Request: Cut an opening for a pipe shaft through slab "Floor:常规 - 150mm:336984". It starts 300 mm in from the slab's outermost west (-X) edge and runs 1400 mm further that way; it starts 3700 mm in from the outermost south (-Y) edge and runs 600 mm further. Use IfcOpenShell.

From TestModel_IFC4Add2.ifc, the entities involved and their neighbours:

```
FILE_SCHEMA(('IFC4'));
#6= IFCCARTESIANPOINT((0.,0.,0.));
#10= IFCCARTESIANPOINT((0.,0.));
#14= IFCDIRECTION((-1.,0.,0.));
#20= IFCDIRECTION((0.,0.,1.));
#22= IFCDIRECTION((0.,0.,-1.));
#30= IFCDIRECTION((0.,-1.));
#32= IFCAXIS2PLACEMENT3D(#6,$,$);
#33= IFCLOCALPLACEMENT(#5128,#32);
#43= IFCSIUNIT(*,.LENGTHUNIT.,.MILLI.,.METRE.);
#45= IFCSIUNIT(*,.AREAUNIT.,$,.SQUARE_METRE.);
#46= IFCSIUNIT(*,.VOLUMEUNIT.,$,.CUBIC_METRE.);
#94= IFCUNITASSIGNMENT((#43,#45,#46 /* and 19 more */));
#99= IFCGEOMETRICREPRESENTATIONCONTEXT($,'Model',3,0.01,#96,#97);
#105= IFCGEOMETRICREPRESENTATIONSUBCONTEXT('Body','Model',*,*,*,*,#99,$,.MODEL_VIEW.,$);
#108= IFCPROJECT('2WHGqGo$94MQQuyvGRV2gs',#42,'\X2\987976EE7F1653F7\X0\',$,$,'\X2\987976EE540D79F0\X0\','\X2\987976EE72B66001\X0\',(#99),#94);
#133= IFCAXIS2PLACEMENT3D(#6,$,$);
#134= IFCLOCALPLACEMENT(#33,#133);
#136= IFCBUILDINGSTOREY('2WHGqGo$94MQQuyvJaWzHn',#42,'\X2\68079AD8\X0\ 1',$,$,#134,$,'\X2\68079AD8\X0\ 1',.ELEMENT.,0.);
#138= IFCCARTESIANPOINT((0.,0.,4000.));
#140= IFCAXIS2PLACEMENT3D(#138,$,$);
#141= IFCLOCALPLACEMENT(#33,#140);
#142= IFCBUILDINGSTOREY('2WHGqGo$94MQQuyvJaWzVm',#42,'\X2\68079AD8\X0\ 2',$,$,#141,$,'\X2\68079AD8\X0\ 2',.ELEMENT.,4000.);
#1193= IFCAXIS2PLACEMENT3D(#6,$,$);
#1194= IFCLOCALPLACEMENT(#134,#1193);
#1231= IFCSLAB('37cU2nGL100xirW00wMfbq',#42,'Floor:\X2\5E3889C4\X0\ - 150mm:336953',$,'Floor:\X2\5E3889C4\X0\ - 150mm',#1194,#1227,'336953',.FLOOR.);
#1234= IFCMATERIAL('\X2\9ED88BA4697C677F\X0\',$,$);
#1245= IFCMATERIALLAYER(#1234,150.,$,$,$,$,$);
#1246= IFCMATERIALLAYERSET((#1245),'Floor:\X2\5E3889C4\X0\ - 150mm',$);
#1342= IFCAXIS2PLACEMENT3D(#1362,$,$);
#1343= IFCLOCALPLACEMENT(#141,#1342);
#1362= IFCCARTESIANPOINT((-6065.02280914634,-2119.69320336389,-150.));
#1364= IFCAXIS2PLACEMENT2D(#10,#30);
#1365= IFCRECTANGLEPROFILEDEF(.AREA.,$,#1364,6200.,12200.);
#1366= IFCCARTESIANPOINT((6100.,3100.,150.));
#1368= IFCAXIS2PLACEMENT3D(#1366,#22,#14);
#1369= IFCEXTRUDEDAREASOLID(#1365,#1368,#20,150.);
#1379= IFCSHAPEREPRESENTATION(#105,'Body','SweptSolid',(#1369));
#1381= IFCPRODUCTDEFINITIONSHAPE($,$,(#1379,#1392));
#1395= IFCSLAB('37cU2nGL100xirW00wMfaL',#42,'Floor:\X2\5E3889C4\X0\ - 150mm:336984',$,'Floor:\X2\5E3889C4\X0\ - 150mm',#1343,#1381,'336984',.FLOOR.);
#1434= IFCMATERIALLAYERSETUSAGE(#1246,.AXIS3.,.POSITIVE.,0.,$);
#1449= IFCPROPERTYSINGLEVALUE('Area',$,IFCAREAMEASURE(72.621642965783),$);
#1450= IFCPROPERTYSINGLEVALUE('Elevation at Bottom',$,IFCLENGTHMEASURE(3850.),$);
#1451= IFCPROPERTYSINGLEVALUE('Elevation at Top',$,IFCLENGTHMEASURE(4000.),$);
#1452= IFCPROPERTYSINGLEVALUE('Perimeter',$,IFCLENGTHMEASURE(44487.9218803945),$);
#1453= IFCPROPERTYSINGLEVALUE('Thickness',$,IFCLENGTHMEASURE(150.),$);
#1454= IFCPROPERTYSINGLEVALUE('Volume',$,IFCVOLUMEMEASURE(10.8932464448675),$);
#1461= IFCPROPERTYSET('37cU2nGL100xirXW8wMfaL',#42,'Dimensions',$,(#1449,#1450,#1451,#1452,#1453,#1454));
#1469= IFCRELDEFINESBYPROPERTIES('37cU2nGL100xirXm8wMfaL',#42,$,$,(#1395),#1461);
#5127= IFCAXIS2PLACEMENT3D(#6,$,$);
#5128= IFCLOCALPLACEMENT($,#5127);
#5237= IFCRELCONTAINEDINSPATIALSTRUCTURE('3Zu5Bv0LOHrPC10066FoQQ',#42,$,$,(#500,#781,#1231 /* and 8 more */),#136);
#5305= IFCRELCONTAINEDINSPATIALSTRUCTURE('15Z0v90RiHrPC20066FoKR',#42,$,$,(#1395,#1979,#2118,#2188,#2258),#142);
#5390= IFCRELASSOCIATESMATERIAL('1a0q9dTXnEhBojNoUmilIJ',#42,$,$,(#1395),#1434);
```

```python
import numpy as np
import ifcopenshell
import ifcopenshell.api.feature
import ifcopenshell.api.geometry
import ifcopenshell.api.pset
import ifcopenshell.api.root
import ifcopenshell.geom
import ifcopenshell.util.element
import ifcopenshell.util.placement
import ifcopenshell.util.representation
import ifcopenshell.util.shape
import ifcopenshell.util.unit

model = ifcopenshell.open("TestModel_IFC4Add2.ifc")
unit_scale = ifcopenshell.util.unit.calculate_unit_scale(model)
area_scale = ifcopenshell.util.unit.calculate_unit_scale(model, "AREAUNIT")
volume_scale = ifcopenshell.util.unit.calculate_unit_scale(model, "VOLUMEUNIT")
settings = ifcopenshell.geom.settings()


def volume(element):
    """Net volume in cubic metres, openings subtracted."""
    shape = ifcopenshell.geom.create_shape(settings, element)
    return ifcopenshell.util.shape.get_volume(shape.geometry)


slab = model.by_guid("37cU2nGL100xirW00wMfaL")
before = volume(slab)

# Extent in the slab's own axes, in metres. The edges named are its -X and -Y sides.
slab_shape = ifcopenshell.geom.create_shape(settings, slab)
vertices = ifcopenshell.util.shape.get_vertices(slab_shape.geometry)
x_min, y_min, bottom = vertices.min(axis=0)
top = vertices[:, 2].max()

opening = ifcopenshell.api.root.create_entity(model, ifc_class="IfcOpeningElement", name="Pipe shaft opening", predefined_type="OPENING")
context = ifcopenshell.util.representation.get_context(model, "Model", "Body", "MODEL_VIEW")
width, depth = 1.4, 0.6
outline = [(0.0, 0.0), (width, 0.0), (width, depth), (0.0, depth), (0.0, 0.0)]
# Overshoot both faces by 50 mm so the cut is clean.
shape = ifcopenshell.api.geometry.add_slab_representation(
    model, context=context, depth=top - bottom + 0.1, polyline=outline
)
ifcopenshell.api.geometry.assign_representation(model, product=opening, representation=shape)

matrix = ifcopenshell.util.placement.get_local_placement(slab.ObjectPlacement)
matrix[:, 3] = matrix @ np.append(np.array([x_min + 0.3, y_min + 3.7, bottom - 0.05]) / unit_scale, 1.0)
ifcopenshell.api.geometry.edit_object_placement(model, product=opening, matrix=matrix, is_si=False)
ifcopenshell.api.feature.add_feature(model, feature=opening, element=slab)

after = volume(slab)

# Update the slab's stored quantities.
pset = model.by_id(ifcopenshell.util.element.get_pset(slab, "Dimensions", should_inherit=False)["id"])
ifcopenshell.api.pset.edit_pset(model, pset=pset, properties={
    "Area": model.create_entity("IfcAreaMeasure", after / (top - bottom) / area_scale),
    "Volume": model.create_entity("IfcVolumeMeasure", after / volume_scale),
})

print(f"slab volume {before:.3f} -> {after:.3f} m3")

model.write("TestModel_IFC4Add2_rev.ifc")
```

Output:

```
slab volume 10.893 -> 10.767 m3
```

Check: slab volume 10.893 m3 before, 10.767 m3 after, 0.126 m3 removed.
